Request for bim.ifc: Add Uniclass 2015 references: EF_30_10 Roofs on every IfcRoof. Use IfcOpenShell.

First a look at what the model holds.

```python
import ifcopenshell

model = ifcopenshell.open("bim.ifc")
print(model.schema)
print("classifications:", [c.Name for c in model.by_type("IfcClassification")])
for ifc_class in ("IfcDoor", "IfcRoof", "IfcStair", "IfcWall", "IfcWindow"):
    print(ifc_class, len(model.by_type(ifc_class)))
```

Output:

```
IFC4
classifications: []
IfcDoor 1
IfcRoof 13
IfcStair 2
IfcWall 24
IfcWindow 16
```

```python
import ifcopenshell
import ifcopenshell.api.classification

model = ifcopenshell.open("bim.ifc")

system = ifcopenshell.api.classification.add_classification(model, classification="Uniclass 2015")

codes = {
    "IfcRoof": ("EF_30_10", "Roofs"),
}
for ifc_class, (code, name) in codes.items():
    products = model.by_type(ifc_class)
    ifcopenshell.api.classification.add_reference(
        model, products=products, classification=system, identification=code, name=name
    )
    print(code, len(products))

model.write("bim_updated.ifc")
```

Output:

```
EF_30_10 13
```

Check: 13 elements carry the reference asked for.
